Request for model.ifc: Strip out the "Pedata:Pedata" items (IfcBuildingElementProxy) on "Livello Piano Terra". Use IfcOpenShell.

First a look at what the model holds.

```python
import ifcopenshell
import ifcopenshell.util.element

model = ifcopenshell.open("model.ifc")
print(model.schema)
storey = next(s for s in model.by_type("IfcBuildingStorey") if s.Name == "Livello Piano Terra")
proxies = [e for e in ifcopenshell.util.element.get_decomposition(storey) if e.is_a("IfcBuildingElementProxy")]
seen = {}
for e in proxies:
    element_type = ifcopenshell.util.element.get_type(e)
    name = element_type.Name if element_type not in (None, e) else None
    seen[name] = seen.get(name, 0) + 1
for name, count in sorted(seen.items(), key=str):
    print(count, "x", name)
```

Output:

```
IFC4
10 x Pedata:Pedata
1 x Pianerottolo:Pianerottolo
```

```python
import ifcopenshell
import ifcopenshell.api.root
import ifcopenshell.util.element

model = ifcopenshell.open("model.ifc")

storey = next(s for s in model.by_type("IfcBuildingStorey") if s.Name == "Livello Piano Terra")
proxies = [e for e in ifcopenshell.util.element.get_decomposition(storey) if e.is_a("IfcBuildingElementProxy")]
targets = [e for e in proxies if (t := ifcopenshell.util.element.get_type(e)) not in (None, e) and t.Name == "Pedata:Pedata"]

for e in targets:
    ifcopenshell.api.root.remove_product(model, product=e)
print(len(targets), "removed")

model.write("model_rev.ifc")
```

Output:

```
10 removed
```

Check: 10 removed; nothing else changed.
